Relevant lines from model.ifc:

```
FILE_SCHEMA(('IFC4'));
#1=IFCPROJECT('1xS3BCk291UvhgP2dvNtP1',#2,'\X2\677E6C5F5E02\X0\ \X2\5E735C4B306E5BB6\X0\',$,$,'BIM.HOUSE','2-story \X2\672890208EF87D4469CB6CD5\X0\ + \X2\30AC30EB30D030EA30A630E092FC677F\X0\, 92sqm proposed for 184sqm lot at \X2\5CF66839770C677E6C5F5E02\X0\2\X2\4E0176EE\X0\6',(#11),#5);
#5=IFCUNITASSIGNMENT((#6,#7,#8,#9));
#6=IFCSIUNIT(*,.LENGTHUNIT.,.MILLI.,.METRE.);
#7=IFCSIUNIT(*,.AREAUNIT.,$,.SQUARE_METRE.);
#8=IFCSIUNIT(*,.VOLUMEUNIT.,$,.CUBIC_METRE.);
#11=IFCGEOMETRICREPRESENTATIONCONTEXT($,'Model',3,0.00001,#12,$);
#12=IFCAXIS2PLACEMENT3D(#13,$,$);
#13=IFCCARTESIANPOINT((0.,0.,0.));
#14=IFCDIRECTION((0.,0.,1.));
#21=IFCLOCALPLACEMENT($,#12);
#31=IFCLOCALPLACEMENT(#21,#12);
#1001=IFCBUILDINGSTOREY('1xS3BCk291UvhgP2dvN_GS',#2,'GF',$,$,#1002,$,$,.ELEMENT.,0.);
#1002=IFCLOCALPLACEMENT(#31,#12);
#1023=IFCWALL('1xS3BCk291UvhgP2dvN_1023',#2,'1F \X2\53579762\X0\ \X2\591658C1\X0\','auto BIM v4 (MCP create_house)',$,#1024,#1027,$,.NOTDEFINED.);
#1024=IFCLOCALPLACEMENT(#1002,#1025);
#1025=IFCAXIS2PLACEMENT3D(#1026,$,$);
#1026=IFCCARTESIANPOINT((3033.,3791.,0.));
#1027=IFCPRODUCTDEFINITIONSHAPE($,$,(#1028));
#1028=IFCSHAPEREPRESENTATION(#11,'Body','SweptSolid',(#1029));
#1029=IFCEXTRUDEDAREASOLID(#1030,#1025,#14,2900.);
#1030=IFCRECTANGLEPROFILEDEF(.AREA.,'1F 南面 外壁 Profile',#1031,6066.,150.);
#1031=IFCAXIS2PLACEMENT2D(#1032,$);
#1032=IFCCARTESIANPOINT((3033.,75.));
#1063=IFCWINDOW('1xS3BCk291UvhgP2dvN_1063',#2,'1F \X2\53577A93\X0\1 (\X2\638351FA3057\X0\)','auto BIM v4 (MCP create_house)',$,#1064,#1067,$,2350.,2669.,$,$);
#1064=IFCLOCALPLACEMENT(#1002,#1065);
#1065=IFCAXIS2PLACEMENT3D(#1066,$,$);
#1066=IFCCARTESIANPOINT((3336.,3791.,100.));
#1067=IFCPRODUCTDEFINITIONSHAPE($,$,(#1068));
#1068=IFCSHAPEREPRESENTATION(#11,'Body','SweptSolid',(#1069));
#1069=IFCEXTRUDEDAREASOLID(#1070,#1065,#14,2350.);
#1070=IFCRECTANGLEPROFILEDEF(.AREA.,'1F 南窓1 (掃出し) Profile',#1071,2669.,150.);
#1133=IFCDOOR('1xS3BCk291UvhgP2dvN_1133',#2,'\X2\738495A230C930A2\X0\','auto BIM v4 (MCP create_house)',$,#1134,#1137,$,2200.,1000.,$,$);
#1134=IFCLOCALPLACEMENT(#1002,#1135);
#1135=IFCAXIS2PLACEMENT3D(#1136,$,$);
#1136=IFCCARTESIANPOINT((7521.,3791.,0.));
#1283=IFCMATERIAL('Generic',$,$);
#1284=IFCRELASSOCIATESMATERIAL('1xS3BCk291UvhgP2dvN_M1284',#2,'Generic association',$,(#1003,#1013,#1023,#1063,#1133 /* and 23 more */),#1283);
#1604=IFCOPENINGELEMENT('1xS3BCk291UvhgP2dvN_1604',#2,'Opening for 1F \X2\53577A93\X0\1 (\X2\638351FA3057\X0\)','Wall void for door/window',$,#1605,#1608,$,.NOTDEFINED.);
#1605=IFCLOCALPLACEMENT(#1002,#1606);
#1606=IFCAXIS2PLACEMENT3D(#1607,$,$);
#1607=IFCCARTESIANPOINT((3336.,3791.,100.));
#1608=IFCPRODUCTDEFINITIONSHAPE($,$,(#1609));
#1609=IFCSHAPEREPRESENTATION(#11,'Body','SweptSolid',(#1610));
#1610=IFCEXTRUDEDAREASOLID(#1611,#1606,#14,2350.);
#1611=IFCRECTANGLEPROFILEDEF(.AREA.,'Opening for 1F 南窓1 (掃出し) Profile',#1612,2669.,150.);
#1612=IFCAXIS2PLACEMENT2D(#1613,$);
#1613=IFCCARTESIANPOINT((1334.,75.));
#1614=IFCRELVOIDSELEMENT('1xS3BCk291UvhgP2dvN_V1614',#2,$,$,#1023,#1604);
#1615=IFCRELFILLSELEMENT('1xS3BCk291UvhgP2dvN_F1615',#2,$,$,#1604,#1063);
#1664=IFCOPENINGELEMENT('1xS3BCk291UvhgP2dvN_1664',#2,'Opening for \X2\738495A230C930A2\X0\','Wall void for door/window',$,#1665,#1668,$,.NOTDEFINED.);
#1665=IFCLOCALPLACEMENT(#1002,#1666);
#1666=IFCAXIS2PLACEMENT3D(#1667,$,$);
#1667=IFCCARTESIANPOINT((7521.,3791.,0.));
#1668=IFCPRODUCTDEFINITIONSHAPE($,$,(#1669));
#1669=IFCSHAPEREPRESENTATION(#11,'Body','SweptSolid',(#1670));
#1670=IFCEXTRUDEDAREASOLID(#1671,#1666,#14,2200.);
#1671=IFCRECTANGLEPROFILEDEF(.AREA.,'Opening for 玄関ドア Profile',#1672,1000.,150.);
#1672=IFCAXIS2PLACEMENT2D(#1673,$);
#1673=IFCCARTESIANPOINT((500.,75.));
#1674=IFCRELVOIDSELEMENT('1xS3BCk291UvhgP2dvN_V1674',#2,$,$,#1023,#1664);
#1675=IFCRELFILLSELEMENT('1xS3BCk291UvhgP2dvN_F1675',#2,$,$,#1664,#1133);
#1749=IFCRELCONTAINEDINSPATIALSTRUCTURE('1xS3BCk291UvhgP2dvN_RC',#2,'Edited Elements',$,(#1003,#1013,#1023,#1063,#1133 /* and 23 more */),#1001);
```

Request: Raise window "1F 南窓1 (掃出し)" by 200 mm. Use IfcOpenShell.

```python
import numpy as np
import ifcopenshell
import ifcopenshell.api.geometry
import ifcopenshell.util.placement
import ifcopenshell.util.unit

model = ifcopenshell.open("model.ifc")
unit_scale = ifcopenshell.util.unit.calculate_unit_scale(model)

window = model.by_id(1063)
opening = window.FillsVoids[0].RelatingOpeningElement
dz = 0.2 / unit_scale

shift = np.array([0.0, 0.0, dz])
# The window is not placed relative to its opening, so move both.
for product in (opening, window):
    matrix = ifcopenshell.util.placement.get_local_placement(product.ObjectPlacement)
    matrix[:3, 3] += shift
    ifcopenshell.api.geometry.edit_object_placement(model, product=product, matrix=matrix, is_si=False)

print(f"moved by {dz * unit_scale:+.3f} m")

model.write("model_rev.ifc")
```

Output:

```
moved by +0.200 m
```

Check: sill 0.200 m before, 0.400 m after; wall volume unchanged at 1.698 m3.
